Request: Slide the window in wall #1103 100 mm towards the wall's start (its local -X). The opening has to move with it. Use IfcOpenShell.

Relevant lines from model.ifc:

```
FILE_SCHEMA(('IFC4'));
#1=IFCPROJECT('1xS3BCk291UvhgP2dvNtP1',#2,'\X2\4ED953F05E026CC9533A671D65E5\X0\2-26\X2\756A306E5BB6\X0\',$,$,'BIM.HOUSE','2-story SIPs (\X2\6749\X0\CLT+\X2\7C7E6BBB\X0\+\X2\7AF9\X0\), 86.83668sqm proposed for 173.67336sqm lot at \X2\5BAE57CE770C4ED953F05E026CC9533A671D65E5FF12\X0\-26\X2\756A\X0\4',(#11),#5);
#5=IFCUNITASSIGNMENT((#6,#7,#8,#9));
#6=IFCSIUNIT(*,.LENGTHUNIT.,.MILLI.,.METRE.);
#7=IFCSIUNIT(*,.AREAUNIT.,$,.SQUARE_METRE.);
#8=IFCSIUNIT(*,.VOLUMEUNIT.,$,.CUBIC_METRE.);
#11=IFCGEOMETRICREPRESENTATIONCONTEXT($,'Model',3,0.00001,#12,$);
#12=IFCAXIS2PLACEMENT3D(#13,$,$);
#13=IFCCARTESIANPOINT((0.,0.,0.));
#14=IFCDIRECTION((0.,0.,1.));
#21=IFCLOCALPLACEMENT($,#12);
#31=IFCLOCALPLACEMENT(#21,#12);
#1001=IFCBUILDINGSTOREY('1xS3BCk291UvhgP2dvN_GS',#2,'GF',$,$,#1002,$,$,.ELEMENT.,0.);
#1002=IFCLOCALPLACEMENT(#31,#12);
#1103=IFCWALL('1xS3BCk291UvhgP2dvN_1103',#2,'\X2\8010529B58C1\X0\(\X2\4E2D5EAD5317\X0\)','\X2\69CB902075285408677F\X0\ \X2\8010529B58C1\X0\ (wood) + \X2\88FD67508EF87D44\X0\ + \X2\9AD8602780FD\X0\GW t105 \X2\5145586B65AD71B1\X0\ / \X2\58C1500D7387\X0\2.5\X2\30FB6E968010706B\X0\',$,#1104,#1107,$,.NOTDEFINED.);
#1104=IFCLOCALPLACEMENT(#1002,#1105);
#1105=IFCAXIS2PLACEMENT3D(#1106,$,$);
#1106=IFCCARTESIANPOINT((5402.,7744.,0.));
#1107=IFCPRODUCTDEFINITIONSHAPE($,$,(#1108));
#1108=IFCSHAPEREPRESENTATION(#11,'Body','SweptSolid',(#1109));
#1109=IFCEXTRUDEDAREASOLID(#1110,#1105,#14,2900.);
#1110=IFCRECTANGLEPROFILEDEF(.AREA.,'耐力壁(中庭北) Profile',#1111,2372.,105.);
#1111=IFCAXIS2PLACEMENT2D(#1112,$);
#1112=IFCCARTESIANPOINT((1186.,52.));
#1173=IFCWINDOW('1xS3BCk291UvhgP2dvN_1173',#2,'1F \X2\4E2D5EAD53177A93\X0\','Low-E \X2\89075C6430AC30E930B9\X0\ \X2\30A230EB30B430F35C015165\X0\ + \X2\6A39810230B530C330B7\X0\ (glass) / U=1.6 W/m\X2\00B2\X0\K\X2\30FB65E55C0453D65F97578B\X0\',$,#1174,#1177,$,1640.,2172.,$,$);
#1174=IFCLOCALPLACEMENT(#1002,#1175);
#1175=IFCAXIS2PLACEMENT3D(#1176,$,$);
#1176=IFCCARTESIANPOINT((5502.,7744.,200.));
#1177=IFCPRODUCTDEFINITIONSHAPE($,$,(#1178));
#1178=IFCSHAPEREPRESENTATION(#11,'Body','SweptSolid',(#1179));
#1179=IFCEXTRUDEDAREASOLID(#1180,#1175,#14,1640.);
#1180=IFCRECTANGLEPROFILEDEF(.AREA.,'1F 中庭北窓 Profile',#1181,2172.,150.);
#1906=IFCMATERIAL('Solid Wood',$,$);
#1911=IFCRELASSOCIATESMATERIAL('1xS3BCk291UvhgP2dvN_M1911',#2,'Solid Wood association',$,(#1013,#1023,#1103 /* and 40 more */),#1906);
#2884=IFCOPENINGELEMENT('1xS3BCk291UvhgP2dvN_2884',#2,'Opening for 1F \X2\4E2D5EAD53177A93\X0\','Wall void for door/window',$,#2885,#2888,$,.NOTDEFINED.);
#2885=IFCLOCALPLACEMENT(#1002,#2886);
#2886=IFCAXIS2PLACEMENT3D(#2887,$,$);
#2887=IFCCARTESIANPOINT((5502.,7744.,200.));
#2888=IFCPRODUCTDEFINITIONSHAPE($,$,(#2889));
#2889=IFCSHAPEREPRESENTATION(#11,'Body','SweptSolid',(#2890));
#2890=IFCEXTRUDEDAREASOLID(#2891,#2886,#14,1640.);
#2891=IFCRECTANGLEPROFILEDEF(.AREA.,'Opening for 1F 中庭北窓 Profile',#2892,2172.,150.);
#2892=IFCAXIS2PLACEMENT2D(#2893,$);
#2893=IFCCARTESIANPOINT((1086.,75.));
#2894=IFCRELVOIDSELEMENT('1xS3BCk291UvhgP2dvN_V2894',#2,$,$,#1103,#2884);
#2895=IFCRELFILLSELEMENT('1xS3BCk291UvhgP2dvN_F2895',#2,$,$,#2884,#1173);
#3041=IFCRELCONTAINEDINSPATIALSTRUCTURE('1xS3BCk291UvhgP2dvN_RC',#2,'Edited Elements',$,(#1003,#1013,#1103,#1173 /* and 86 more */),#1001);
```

```python
import ifcopenshell
import ifcopenshell.api.geometry
import ifcopenshell.util.placement
import ifcopenshell.util.unit

model = ifcopenshell.open("model.ifc")
unit_scale = ifcopenshell.util.unit.calculate_unit_scale(model)

window = model.by_guid("1xS3BCk291UvhgP2dvN_1173")
opening = window.FillsVoids[0].RelatingOpeningElement
wall = opening.VoidsElements[0].RelatingBuildingElement

wall_matrix = ifcopenshell.util.placement.get_local_placement(wall.ObjectPlacement)
shift = wall_matrix[:3, 0] * -0.1 / unit_scale
before = ifcopenshell.util.placement.get_local_placement(window.ObjectPlacement)[:3, 3].copy()

# The window is not placed relative to its opening, so move both.
for product in (opening, window):
    matrix = ifcopenshell.util.placement.get_local_placement(product.ObjectPlacement)
    matrix[:3, 3] += shift
    ifcopenshell.api.geometry.edit_object_placement(model, product=product, matrix=matrix, is_si=False)

after = ifcopenshell.util.placement.get_local_placement(window.ObjectPlacement)[:3, 3]
print("window moved by", (after - before).round(3) + 0.0)

model.write("model-out.ifc")
```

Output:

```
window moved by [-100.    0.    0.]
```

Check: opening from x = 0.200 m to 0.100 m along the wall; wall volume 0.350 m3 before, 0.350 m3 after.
